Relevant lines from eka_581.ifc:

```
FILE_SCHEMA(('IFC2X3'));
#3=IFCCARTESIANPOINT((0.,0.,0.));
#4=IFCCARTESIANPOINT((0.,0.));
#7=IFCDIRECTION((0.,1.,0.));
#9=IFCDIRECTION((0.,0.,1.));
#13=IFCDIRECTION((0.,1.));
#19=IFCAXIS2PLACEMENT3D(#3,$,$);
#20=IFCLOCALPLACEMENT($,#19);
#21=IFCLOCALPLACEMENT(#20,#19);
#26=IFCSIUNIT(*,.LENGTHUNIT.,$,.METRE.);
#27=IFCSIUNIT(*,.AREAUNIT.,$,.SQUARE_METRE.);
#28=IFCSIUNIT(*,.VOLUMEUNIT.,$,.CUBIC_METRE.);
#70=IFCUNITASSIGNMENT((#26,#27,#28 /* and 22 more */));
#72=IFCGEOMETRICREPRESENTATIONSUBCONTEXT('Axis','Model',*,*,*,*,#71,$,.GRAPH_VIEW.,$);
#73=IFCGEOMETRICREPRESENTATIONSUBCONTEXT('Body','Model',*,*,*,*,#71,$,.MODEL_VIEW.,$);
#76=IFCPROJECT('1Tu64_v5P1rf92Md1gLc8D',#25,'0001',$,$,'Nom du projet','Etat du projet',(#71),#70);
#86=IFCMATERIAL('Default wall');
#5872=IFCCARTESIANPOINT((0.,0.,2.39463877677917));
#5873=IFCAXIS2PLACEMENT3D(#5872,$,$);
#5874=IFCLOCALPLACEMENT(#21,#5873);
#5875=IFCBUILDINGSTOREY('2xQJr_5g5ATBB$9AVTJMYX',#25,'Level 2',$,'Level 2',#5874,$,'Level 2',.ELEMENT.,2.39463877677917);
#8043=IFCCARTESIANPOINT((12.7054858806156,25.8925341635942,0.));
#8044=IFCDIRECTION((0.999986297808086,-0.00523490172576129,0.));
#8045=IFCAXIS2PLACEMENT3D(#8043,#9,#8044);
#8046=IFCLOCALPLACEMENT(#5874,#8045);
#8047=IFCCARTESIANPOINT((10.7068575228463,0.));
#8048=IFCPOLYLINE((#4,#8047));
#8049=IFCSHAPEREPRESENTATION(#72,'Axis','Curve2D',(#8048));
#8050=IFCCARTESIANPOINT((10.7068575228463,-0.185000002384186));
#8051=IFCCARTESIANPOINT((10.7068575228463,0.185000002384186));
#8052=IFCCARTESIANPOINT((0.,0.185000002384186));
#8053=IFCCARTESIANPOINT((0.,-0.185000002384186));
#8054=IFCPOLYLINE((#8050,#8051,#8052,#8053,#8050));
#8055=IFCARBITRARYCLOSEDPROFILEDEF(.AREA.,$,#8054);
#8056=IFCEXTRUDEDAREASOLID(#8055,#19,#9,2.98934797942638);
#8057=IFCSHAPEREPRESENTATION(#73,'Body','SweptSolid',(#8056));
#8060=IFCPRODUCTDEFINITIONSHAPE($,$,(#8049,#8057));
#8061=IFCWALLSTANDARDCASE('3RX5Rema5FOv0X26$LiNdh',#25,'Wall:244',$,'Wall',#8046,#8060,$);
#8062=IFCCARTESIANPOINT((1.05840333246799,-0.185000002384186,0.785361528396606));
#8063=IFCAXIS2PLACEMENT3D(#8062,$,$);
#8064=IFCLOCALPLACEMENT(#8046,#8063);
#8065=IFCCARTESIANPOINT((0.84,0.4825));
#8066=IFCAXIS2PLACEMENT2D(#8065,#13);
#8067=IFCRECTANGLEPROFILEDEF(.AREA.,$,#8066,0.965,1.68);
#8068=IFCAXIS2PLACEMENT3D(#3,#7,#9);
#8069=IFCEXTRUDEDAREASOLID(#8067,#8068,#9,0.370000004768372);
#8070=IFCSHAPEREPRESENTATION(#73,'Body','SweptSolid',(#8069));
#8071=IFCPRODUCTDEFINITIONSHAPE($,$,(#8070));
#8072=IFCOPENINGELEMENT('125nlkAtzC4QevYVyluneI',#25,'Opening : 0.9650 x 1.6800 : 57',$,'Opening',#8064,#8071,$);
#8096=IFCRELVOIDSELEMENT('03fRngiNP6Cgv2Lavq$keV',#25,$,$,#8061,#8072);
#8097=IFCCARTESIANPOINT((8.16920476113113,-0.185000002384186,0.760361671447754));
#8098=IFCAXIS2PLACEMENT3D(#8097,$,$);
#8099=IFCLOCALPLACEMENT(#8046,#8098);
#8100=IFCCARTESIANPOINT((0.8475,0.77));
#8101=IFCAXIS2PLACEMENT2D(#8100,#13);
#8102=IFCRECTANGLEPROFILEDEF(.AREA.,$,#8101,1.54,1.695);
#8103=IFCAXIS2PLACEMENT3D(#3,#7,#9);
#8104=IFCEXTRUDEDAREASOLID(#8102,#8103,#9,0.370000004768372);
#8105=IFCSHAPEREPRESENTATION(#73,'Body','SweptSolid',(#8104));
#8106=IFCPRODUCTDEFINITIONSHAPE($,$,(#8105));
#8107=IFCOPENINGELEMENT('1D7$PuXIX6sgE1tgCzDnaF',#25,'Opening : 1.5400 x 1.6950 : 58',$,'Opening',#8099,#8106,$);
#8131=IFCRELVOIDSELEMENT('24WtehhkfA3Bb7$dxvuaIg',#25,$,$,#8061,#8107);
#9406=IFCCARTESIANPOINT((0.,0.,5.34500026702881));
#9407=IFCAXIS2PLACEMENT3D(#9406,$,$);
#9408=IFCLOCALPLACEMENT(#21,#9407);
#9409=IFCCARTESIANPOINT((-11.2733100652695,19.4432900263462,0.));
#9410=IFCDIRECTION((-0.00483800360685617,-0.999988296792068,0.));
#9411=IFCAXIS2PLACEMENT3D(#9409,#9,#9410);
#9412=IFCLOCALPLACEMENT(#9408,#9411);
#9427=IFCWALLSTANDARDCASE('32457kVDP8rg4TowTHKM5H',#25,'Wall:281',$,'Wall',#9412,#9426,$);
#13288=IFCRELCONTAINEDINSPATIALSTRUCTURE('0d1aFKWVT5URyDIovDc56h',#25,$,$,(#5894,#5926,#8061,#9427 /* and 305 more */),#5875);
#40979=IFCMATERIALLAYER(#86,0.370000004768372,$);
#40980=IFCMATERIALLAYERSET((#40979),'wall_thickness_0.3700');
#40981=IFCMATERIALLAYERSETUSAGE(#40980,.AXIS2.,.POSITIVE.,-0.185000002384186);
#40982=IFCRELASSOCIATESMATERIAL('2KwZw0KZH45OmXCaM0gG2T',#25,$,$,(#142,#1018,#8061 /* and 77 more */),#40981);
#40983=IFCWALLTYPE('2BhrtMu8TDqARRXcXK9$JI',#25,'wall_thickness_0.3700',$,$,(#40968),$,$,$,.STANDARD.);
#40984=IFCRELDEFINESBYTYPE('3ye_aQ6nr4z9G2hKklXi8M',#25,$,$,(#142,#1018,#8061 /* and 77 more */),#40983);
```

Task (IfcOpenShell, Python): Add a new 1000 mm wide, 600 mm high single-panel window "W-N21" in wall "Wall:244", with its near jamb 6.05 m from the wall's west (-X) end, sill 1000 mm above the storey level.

```python
import numpy as np
import ifcopenshell
import ifcopenshell.api.feature
import ifcopenshell.api.geometry
import ifcopenshell.api.root
import ifcopenshell.api.spatial
import ifcopenshell.api.type
import ifcopenshell.geom
import ifcopenshell.util.element
import ifcopenshell.util.placement
import ifcopenshell.util.representation
import ifcopenshell.util.shape
import ifcopenshell.util.unit

model = ifcopenshell.open("eka_581.ifc")
unit_scale = ifcopenshell.util.unit.calculate_unit_scale(model)
settings = ifcopenshell.geom.settings()


def volume(element):
    """Net volume in cubic metres, openings subtracted."""
    shape = ifcopenshell.geom.create_shape(settings, element)
    return ifcopenshell.util.shape.get_volume(shape.geometry)


wall = model.by_guid("3RX5Rema5FOv0X26$LiNdh")
storey = ifcopenshell.util.element.get_container(wall, ifc_class="IfcBuildingStorey")
context = ifcopenshell.util.representation.get_context(model, "Model", "Body", "MODEL_VIEW")
before = volume(wall)

width, height, from_end, sill = 1, 0.6, 6.05, 1  # metres

# The wall runs along its own X axis, and the end named is its -X end.
wall_shape = ifcopenshell.geom.create_shape(settings, wall)
x, y, z = ifcopenshell.util.shape.get_vertices(wall_shape.geometry).T
start = x.min() + from_end
face, thickness = float(y.min()), float(y.max() - y.min())
wall_matrix = ifcopenshell.util.placement.get_local_placement(wall.ObjectPlacement)
level = ifcopenshell.util.placement.get_local_placement(storey.ObjectPlacement)[2, 3]


def in_wall(x, y):
    """Placement at x, y metres in the wall's axes, at sill height."""
    matrix = wall_matrix.copy()
    matrix[:, 3] = wall_matrix @ np.array([x / unit_scale, y / unit_scale, 0.0, 1.0])
    matrix[2, 3] = level + sill / unit_scale
    return matrix


# Opening: a box that overshoots both wall faces by 50 mm.
opening = ifcopenshell.api.root.create_entity(model, ifc_class="IfcOpeningElement")
box = ifcopenshell.api.geometry.add_wall_representation(
    model, context=context, length=width, height=height, thickness=thickness + 0.1
)
ifcopenshell.api.geometry.assign_representation(model, product=opening, representation=box)
ifcopenshell.api.geometry.edit_object_placement(model, product=opening, matrix=in_wall(start, face - 0.05), is_si=False)
ifcopenshell.api.feature.add_feature(model, feature=opening, element=wall)

window = ifcopenshell.api.root.create_entity(model, ifc_class="IfcWindow", name="W-N21")
window.OverallWidth, window.OverallHeight = width / unit_scale, height / unit_scale
body = ifcopenshell.api.geometry.add_window_representation(
    model,
    context=context,
    overall_width=window.OverallWidth,
    overall_height=window.OverallHeight,
    partition_type="SINGLE_PANEL",
)
ifcopenshell.api.geometry.assign_representation(model, product=window, representation=body)
ifcopenshell.api.spatial.assign_container(model, products=[window], relating_structure=storey)
fills = ifcopenshell.api.feature.add_filling(model, opening=opening, element=window)
fills.OwnerHistory = window.OwnerHistory  # required in IFC2X3

# IFC2X3 keeps the operation on the window style.
style = ifcopenshell.api.root.create_entity(model, ifc_class="IfcWindowStyle", name="W-N21")
style.OperationType, style.ConstructionType = "SINGLE_PANEL", "NOTDEFINED"
style.ParameterTakesPrecedence = style.Sizeable = False
ifcopenshell.api.type.assign_type(model, related_objects=[window], relating_type=style)

# Centre the window in the wall's thickness.
ifcopenshell.api.geometry.edit_object_placement(model, product=window, matrix=in_wall(start, face), is_si=False)
window_shape = ifcopenshell.geom.create_shape(settings, window)
depth = ifcopenshell.util.shape.get_vertices(window_shape.geometry)[:, 1]
offset = face + thickness / 2 - (depth.min() + depth.max()) / 2
ifcopenshell.api.geometry.edit_object_placement(model, product=window, matrix=in_wall(start, offset), is_si=False)

after = volume(wall)

print(f"wall volume {before:.3f} -> {after:.3f} m3")

model.write("eka_581_edited.ifc")
```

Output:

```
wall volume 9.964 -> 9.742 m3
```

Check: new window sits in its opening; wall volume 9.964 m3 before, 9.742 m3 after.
